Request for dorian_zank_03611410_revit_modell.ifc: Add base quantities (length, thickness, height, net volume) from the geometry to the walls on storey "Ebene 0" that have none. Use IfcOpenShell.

First a look at what the model holds.

```python
import ifcopenshell
import ifcopenshell.util.element
import ifcopenshell.util.unit

model = ifcopenshell.open("dorian_zank_03611410_revit_modell.ifc")
print(model.schema)
for unit_type in ("LENGTHUNIT", "AREAUNIT", "VOLUMEUNIT"):
    print(unit_type, ifcopenshell.util.unit.calculate_unit_scale(model, unit_type))
storey = next(s for s in model.by_type("IfcBuildingStorey") if s.Name == "Ebene 0")
walls = [e for e in ifcopenshell.util.element.get_decomposition(storey) if e.is_a("IfcWall")]
for e in sorted(walls, key=lambda e: e.id()):
    print(e.id(), e.is_a(), e.Name, list(ifcopenshell.util.element.get_psets(e, qtos_only=True)), sep=" | ")
```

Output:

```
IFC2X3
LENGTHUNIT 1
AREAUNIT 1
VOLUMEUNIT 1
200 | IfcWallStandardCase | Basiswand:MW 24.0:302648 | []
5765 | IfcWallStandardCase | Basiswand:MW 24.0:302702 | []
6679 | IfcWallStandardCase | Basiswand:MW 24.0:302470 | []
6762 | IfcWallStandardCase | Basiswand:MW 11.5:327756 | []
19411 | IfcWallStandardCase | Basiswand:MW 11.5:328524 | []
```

```python
import ifcopenshell
import ifcopenshell.api.pset
import ifcopenshell.geom
import ifcopenshell.util.element
import ifcopenshell.util.shape
import ifcopenshell.util.unit

model = ifcopenshell.open("dorian_zank_03611410_revit_modell.ifc")
unit_scale = ifcopenshell.util.unit.calculate_unit_scale(model)
volume_scale = ifcopenshell.util.unit.calculate_unit_scale(model, "VOLUMEUNIT")
settings = ifcopenshell.geom.settings()

storey = next(s for s in model.by_type("IfcBuildingStorey") if s.Name == "Ebene 0")
walls = [e for e in ifcopenshell.util.element.get_decomposition(storey) if e.is_a("IfcWall")]

for e in sorted(walls, key=lambda e: e.id()):
    if ifcopenshell.util.element.get_psets(e, qtos_only=True, should_inherit=False):
        continue
    # Geometry comes back in metres, in the element's own axes.
    shape = ifcopenshell.geom.create_shape(settings, e)
    values = {
        "Length": ifcopenshell.util.shape.get_x(shape.geometry) / unit_scale,
        "Width": ifcopenshell.util.shape.get_y(shape.geometry) / unit_scale,
        "Height": ifcopenshell.util.shape.get_z(shape.geometry) / unit_scale,
        "NetVolume": ifcopenshell.util.shape.get_volume(shape.geometry) / volume_scale,
    }
    qto = ifcopenshell.api.pset.add_qto(model, product=e, name="BaseQuantities")
    ifcopenshell.api.pset.edit_qto(model, qto=qto, properties=values)
    print(e.id(), {k: round(v, 3) for k, v in values.items()})

model.write("dorian_zank_03611410_revit_modell_v2.ifc")
```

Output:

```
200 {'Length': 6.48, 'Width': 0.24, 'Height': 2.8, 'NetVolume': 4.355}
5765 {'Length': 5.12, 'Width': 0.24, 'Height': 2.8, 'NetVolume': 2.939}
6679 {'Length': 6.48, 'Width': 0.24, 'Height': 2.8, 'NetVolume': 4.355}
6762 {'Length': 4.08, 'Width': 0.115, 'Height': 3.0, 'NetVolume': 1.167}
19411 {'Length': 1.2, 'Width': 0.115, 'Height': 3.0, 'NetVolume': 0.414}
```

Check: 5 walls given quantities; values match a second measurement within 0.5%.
